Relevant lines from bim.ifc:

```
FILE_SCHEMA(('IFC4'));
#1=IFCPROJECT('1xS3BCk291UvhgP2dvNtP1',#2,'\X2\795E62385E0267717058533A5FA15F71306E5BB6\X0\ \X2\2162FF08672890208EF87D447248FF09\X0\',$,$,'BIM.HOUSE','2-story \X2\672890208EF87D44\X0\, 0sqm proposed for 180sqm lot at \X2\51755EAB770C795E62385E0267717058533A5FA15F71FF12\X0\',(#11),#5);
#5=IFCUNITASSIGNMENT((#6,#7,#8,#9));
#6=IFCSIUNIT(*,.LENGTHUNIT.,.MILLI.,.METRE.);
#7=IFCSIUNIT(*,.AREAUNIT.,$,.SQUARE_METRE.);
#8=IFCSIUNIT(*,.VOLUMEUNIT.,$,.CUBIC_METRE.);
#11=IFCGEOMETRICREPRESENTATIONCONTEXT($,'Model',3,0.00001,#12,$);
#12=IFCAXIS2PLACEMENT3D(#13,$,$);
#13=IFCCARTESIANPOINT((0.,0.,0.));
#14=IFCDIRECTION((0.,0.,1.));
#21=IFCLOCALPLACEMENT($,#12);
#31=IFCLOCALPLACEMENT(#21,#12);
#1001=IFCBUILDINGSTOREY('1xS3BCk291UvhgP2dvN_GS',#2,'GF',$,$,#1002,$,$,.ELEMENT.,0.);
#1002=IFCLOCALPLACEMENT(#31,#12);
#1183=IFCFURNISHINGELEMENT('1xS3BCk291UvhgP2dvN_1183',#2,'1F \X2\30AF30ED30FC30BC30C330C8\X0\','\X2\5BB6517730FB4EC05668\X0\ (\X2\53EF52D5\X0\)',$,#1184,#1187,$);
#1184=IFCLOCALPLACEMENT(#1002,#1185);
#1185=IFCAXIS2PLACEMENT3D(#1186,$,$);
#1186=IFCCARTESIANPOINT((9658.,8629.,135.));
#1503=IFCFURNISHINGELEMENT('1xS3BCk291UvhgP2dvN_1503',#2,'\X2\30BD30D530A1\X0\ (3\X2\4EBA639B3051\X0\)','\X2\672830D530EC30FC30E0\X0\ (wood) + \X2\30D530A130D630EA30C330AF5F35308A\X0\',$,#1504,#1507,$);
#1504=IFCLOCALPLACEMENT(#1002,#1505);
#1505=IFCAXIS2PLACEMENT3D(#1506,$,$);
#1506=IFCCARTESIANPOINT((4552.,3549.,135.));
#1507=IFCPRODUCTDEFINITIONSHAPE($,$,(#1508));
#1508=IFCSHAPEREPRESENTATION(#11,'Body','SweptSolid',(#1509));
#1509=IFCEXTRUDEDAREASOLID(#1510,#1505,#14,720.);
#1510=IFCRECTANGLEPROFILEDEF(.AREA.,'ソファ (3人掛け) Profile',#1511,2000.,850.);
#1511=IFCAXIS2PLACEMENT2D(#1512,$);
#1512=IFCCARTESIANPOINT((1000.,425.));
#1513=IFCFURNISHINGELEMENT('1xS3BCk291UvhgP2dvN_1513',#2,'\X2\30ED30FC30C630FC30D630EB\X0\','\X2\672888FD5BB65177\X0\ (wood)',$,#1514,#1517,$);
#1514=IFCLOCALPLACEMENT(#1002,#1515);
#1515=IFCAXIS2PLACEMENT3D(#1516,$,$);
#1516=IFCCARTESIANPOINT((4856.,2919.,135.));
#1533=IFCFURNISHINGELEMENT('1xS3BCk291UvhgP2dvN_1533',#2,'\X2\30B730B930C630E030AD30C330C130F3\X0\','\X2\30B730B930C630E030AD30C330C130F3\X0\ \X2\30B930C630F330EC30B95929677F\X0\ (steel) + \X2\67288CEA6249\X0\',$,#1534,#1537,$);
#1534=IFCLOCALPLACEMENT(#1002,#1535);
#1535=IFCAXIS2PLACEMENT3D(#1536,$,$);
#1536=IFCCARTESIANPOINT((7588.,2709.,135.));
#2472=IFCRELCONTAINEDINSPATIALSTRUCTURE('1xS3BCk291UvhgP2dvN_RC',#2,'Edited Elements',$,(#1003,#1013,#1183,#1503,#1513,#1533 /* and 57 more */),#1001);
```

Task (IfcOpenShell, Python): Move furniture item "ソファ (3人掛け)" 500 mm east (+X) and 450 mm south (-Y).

```python
import ifcopenshell
import ifcopenshell.api.geometry
import ifcopenshell.util.placement
import ifcopenshell.util.unit

model = ifcopenshell.open("bim.ifc")
unit_scale = ifcopenshell.util.unit.calculate_unit_scale(model)

item = model.by_guid("1xS3BCk291UvhgP2dvN_1503")
matrix = ifcopenshell.util.placement.get_local_placement(item.ObjectPlacement)
matrix[0, 3] += 0.5 / unit_scale
matrix[1, 3] -= 0.45 / unit_scale
ifcopenshell.api.geometry.edit_object_placement(model, product=item, matrix=matrix, is_si=False)

print(ifcopenshell.util.placement.get_local_placement(item.ObjectPlacement).round(3) + 0.0)

model.write("bim_updated.ifc")
```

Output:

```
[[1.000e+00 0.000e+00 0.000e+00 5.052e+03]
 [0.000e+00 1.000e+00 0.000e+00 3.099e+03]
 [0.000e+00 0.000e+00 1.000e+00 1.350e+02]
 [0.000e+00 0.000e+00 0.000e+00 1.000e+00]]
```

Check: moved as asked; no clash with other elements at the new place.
